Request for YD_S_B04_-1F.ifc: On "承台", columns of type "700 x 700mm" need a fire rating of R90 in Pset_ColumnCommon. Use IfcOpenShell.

First a look at what the model holds.

```python
import ifcopenshell
import ifcopenshell.util.element

model = ifcopenshell.open("YD_S_B04_-1F.ifc")
print(model.schema)
storey = next(s for s in model.by_type("IfcBuildingStorey") if s.Name == "承台")
columns = [e for e in ifcopenshell.util.element.get_decomposition(storey) if e.is_a("IfcColumn")]
seen = {}
for e in columns:
    element_type = ifcopenshell.util.element.get_type(e)
    key = (element_type.Name if element_type != e and element_type else None, ifcopenshell.util.element.get_pset(e, "Pset_ColumnCommon", "FireRating"))
    seen[key] = seen.get(key, 0) + 1
for (name, value), count in sorted(seen.items(), key=str):
    print(count, "x", name, "|", value)
```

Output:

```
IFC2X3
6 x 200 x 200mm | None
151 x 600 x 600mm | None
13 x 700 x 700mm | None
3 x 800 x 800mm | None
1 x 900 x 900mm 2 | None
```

```python
import ifcopenshell
import ifcopenshell.api.pset
import ifcopenshell.util.element

model = ifcopenshell.open("YD_S_B04_-1F.ifc")

storey = next(s for s in model.by_type("IfcBuildingStorey") if s.Name == "承台")
columns = [e for e in ifcopenshell.util.element.get_decomposition(storey) if e.is_a("IfcColumn")]

count = 0
for e in columns:
    element_type = ifcopenshell.util.element.get_type(e)
    if element_type in (None, e) or element_type.Name != "700 x 700mm":
        continue
    # add_pset returns the element's existing set when there is one.
    pset = ifcopenshell.api.pset.add_pset(model, product=e, name="Pset_ColumnCommon")
    ifcopenshell.api.pset.edit_pset(model, pset=pset, properties={"FireRating": "R90"})
    count += 1

print(count, "columns updated")

model.write("YD_S_B04_-1F_rev.ifc")
```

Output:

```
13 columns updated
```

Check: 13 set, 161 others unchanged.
